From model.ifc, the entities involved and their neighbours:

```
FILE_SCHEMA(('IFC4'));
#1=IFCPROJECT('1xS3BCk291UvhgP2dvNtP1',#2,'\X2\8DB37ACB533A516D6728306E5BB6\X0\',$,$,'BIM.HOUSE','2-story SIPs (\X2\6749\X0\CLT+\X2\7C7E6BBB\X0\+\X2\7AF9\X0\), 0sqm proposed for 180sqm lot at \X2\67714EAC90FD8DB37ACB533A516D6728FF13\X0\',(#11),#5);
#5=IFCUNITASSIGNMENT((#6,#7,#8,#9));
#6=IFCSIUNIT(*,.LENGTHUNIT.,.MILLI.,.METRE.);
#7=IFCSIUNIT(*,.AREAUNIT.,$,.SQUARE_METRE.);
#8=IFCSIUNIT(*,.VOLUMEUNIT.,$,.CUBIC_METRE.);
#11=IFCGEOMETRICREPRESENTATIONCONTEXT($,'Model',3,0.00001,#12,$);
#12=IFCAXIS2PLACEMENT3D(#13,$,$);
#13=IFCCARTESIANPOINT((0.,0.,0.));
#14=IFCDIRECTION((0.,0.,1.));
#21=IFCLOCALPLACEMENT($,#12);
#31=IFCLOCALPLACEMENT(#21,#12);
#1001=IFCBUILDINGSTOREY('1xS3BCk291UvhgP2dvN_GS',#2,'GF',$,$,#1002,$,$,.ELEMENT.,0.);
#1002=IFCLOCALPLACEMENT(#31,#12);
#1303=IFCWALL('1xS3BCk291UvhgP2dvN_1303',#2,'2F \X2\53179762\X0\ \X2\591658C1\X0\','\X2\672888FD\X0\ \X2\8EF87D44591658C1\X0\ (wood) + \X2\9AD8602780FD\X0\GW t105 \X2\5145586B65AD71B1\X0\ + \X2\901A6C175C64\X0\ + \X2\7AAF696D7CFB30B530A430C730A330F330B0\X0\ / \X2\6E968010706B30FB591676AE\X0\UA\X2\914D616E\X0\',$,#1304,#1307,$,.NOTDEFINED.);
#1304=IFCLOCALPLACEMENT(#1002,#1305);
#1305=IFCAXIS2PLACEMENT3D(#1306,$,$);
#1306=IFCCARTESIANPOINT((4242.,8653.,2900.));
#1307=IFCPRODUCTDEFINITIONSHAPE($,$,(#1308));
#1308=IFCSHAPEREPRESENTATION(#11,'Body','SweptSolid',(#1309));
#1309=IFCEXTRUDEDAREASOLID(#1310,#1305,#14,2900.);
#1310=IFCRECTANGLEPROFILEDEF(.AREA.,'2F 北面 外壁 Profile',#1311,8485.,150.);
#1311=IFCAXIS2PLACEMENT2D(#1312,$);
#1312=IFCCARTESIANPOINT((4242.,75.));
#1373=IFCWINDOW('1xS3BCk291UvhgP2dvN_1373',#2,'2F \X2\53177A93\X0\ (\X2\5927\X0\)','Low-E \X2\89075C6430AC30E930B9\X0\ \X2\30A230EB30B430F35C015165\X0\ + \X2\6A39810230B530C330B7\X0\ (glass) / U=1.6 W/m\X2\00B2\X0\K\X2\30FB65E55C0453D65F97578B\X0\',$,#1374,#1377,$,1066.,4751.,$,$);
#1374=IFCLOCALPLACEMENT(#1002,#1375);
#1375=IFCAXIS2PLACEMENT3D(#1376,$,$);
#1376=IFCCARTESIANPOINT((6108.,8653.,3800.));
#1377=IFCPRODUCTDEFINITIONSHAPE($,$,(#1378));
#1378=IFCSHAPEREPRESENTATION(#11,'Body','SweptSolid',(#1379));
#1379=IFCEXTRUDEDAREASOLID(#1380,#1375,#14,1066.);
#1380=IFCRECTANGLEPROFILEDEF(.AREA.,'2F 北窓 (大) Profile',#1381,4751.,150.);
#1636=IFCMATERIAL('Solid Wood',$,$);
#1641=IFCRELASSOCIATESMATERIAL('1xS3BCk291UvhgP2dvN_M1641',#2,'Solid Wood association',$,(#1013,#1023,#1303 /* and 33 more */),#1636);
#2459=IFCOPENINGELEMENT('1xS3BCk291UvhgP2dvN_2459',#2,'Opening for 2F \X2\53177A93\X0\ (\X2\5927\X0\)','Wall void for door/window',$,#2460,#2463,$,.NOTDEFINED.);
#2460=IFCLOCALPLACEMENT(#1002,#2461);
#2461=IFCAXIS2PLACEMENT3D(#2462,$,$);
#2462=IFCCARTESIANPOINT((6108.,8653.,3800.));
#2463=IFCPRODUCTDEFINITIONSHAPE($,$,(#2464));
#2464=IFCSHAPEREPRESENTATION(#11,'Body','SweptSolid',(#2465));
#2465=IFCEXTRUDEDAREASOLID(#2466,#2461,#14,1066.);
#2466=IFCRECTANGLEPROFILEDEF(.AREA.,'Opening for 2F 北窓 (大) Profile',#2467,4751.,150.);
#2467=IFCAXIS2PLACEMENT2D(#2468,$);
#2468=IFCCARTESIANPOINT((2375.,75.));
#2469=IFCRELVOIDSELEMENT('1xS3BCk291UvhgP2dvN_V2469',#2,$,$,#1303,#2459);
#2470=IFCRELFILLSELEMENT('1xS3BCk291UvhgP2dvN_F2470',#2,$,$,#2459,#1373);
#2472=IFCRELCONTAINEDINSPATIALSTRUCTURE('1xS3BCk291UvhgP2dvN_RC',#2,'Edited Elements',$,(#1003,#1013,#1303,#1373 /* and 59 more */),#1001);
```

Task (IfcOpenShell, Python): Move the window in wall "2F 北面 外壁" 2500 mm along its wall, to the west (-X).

```python
import ifcopenshell
import ifcopenshell.api.geometry
import ifcopenshell.util.placement
import ifcopenshell.util.unit

model = ifcopenshell.open("model.ifc")
unit_scale = ifcopenshell.util.unit.calculate_unit_scale(model)

window = model.by_guid("1xS3BCk291UvhgP2dvN_1373")
opening = window.FillsVoids[0].RelatingOpeningElement
wall = opening.VoidsElements[0].RelatingBuildingElement

wall_matrix = ifcopenshell.util.placement.get_local_placement(wall.ObjectPlacement)
shift = wall_matrix[:3, 0] * -2.5 / unit_scale
before = ifcopenshell.util.placement.get_local_placement(window.ObjectPlacement)[:3, 3].copy()

# The window is not placed relative to its opening, so move both.
for product in (opening, window):
    matrix = ifcopenshell.util.placement.get_local_placement(product.ObjectPlacement)
    matrix[:3, 3] += shift
    ifcopenshell.api.geometry.edit_object_placement(model, product=product, matrix=matrix, is_si=False)

after = ifcopenshell.util.placement.get_local_placement(window.ObjectPlacement)[:3, 3]
print("window moved by", (after - before).round(3) + 0.0)

model.write("model_v2.ifc")
```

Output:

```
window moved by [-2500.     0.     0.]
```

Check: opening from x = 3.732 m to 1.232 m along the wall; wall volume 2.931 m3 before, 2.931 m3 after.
